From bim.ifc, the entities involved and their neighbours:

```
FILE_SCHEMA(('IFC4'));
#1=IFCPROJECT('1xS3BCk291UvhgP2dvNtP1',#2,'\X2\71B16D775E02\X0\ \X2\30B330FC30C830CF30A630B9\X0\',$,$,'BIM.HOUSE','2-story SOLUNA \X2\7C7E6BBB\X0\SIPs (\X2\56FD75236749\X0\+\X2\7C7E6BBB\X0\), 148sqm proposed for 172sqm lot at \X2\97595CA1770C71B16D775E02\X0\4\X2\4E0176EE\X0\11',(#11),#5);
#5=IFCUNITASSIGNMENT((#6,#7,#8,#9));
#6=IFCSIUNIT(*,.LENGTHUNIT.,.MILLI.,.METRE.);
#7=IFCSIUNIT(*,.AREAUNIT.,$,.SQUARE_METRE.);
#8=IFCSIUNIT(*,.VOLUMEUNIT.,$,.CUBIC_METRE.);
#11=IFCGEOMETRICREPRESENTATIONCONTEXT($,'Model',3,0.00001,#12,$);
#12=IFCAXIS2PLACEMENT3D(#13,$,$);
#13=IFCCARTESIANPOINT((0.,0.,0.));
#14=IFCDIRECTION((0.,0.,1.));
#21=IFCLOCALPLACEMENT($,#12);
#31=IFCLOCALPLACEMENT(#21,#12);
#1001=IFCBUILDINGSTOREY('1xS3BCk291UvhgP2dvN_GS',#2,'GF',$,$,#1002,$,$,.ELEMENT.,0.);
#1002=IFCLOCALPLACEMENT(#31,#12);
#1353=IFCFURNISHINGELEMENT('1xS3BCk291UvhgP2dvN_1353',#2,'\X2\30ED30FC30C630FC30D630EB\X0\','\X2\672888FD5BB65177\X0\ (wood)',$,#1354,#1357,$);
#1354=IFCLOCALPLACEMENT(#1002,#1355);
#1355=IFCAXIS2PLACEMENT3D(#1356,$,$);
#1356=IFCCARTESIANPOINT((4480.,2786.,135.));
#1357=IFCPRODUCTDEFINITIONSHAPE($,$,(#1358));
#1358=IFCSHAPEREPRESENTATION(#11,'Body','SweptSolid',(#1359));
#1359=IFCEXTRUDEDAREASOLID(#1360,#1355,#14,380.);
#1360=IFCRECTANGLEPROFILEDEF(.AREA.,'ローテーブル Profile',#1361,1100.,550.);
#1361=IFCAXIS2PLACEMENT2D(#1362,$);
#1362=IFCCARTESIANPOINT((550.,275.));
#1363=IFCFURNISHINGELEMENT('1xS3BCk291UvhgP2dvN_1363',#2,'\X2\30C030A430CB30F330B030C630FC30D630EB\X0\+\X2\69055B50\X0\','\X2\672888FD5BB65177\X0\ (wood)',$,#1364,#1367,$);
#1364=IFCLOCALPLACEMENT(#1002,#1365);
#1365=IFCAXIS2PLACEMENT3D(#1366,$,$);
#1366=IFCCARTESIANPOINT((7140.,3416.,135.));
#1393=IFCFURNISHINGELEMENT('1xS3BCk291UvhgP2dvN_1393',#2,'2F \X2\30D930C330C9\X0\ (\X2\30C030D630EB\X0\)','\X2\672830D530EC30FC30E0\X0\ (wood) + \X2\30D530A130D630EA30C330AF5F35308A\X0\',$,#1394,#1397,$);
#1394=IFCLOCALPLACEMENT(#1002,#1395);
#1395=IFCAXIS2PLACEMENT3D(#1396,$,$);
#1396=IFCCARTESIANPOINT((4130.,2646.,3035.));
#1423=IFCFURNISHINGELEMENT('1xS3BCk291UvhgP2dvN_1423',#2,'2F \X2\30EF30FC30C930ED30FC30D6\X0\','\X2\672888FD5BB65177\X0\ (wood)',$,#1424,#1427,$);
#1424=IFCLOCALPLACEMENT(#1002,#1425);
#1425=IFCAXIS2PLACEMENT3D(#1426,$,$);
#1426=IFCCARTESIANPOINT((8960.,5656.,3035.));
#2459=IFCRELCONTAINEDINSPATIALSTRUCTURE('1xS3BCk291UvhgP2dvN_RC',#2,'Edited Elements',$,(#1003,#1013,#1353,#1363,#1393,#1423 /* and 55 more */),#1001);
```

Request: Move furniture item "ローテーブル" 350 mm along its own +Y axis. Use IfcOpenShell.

```python
import ifcopenshell
import ifcopenshell.api.geometry
import ifcopenshell.util.placement
import ifcopenshell.util.unit

model = ifcopenshell.open("bim.ifc")
unit_scale = ifcopenshell.util.unit.calculate_unit_scale(model)

item = model.by_id(1353)
matrix = ifcopenshell.util.placement.get_local_placement(item.ObjectPlacement)
matrix[:3, 3] += matrix[:3, 1] * 0.35 / unit_scale
ifcopenshell.api.geometry.edit_object_placement(model, product=item, matrix=matrix, is_si=False)

print(ifcopenshell.util.placement.get_local_placement(item.ObjectPlacement).round(3) + 0.0)

model.write("bim_updated.ifc")
```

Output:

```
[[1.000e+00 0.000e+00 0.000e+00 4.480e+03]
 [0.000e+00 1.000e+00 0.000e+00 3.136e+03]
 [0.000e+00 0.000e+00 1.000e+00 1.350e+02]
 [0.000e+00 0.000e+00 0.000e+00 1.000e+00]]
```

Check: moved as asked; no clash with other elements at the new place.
